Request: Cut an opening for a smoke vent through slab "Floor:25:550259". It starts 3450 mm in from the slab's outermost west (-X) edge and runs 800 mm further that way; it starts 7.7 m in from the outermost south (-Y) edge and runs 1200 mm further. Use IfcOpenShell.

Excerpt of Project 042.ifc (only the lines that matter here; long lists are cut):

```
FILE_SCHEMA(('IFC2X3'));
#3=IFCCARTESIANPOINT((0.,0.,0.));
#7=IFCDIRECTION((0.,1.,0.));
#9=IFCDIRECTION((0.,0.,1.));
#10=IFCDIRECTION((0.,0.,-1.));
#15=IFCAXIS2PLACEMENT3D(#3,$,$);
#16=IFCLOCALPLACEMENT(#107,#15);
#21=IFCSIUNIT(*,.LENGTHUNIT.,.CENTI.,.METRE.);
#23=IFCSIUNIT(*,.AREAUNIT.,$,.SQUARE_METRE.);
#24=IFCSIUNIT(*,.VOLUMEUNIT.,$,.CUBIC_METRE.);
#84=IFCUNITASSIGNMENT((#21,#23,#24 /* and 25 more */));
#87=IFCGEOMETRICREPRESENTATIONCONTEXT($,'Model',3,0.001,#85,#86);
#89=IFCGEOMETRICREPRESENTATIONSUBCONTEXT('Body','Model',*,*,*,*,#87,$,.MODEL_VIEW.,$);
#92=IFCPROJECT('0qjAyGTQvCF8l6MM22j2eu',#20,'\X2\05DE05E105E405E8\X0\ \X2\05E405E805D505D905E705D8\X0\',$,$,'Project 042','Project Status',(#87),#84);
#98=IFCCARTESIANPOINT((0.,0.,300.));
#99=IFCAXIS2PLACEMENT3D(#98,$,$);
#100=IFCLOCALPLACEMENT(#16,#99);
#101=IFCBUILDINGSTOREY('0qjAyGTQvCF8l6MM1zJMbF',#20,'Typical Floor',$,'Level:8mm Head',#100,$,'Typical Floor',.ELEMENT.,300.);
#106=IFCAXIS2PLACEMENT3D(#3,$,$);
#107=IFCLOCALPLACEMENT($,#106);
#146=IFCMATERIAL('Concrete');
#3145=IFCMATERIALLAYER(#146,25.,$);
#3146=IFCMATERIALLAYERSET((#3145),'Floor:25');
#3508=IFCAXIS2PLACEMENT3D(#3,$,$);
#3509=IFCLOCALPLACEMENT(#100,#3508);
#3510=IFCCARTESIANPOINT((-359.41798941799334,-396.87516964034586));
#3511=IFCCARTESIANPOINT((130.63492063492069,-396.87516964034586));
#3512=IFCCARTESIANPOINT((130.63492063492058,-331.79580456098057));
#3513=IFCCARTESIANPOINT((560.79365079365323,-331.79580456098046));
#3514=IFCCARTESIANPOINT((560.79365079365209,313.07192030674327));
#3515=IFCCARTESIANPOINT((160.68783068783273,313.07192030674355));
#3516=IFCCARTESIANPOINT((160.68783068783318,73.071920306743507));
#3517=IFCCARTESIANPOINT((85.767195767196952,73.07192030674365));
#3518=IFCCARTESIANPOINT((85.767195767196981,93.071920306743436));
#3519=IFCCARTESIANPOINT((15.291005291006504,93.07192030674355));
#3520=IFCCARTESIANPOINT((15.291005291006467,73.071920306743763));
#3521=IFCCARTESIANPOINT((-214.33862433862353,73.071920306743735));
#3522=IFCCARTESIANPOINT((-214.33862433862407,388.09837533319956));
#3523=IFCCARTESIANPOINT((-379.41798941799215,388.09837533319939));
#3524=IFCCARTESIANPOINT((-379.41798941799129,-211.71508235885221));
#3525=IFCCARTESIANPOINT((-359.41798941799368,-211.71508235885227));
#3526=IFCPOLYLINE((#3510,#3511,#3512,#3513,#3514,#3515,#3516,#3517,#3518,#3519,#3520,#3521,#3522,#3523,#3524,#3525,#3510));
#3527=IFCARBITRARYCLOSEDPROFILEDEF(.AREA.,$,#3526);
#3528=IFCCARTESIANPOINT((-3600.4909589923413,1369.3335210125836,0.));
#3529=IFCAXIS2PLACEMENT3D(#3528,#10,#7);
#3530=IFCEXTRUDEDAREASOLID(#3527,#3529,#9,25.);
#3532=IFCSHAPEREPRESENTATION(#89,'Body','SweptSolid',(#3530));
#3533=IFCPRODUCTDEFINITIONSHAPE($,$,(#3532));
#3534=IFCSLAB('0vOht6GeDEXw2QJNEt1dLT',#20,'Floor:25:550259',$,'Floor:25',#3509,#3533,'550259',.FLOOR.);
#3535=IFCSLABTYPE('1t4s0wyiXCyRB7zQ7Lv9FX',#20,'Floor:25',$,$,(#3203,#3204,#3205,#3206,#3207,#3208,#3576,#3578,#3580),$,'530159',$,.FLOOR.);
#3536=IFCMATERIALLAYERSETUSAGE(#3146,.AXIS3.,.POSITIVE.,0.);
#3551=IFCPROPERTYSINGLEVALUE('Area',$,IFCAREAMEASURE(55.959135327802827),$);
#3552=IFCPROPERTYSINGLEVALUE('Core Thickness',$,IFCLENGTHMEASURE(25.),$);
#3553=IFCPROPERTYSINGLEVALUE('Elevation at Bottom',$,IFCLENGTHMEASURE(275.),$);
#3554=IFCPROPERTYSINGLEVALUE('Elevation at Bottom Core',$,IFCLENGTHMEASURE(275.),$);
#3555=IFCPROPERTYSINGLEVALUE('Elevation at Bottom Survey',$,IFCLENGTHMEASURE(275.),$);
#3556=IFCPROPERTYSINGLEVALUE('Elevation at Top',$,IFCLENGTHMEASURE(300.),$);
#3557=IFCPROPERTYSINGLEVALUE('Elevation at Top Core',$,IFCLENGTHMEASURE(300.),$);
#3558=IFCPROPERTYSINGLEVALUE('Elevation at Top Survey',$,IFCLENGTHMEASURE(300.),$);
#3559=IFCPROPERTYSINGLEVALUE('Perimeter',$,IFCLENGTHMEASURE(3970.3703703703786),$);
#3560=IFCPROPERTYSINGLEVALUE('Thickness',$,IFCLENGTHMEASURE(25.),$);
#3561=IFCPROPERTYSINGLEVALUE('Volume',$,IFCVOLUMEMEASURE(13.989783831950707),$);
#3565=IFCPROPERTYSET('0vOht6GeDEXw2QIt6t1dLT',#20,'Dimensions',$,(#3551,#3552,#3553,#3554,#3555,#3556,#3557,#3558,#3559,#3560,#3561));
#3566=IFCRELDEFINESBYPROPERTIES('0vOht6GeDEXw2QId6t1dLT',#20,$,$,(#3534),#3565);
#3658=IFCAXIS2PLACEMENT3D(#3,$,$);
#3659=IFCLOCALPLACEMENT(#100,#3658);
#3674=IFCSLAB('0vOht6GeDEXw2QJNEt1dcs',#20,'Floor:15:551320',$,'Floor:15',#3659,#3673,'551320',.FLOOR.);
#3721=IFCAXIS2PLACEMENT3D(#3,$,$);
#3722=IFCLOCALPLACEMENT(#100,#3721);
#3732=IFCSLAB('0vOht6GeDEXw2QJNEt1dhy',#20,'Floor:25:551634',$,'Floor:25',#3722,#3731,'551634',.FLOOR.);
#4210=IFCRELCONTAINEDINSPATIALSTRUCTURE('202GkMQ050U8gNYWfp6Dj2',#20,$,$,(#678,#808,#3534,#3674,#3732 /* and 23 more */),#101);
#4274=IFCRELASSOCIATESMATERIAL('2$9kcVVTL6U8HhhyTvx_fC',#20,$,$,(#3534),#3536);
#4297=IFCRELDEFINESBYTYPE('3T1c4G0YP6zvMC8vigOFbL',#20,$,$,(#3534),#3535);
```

```python
import numpy as np
import ifcopenshell
import ifcopenshell.api.feature
import ifcopenshell.api.geometry
import ifcopenshell.api.pset
import ifcopenshell.api.root
import ifcopenshell.geom
import ifcopenshell.util.element
import ifcopenshell.util.placement
import ifcopenshell.util.representation
import ifcopenshell.util.shape
import ifcopenshell.util.unit

model = ifcopenshell.open("Project 042.ifc")
unit_scale = ifcopenshell.util.unit.calculate_unit_scale(model)
area_scale = ifcopenshell.util.unit.calculate_unit_scale(model, "AREAUNIT")
volume_scale = ifcopenshell.util.unit.calculate_unit_scale(model, "VOLUMEUNIT")
settings = ifcopenshell.geom.settings()


def volume(element):
    """Net volume in cubic metres, openings subtracted."""
    shape = ifcopenshell.geom.create_shape(settings, element)
    return ifcopenshell.util.shape.get_volume(shape.geometry)


slab = model.by_guid("0vOht6GeDEXw2QJNEt1dLT")
before = volume(slab)

# Extent in the slab's own axes, in metres. The edges named are its -X and -Y sides.
slab_shape = ifcopenshell.geom.create_shape(settings, slab)
vertices = ifcopenshell.util.shape.get_vertices(slab_shape.geometry)
x_min, y_min, bottom = vertices.min(axis=0)
top = vertices[:, 2].max()

opening = ifcopenshell.api.root.create_entity(model, ifc_class="IfcOpeningElement", name="Smoke vent opening")
context = ifcopenshell.util.representation.get_context(model, "Model", "Body", "MODEL_VIEW")
width, depth = 0.8, 1.2
outline = [(0.0, 0.0), (width, 0.0), (width, depth), (0.0, depth), (0.0, 0.0)]
# Overshoot both faces by 50 mm so the cut is clean.
shape = ifcopenshell.api.geometry.add_slab_representation(
    model, context=context, depth=top - bottom + 0.1, polyline=outline
)
ifcopenshell.api.geometry.assign_representation(model, product=opening, representation=shape)

matrix = ifcopenshell.util.placement.get_local_placement(slab.ObjectPlacement)
matrix[:, 3] = matrix @ np.append(np.array([x_min + 3.45, y_min + 7.7, bottom - 0.05]) / unit_scale, 1.0)
ifcopenshell.api.geometry.edit_object_placement(model, product=opening, matrix=matrix, is_si=False)
ifcopenshell.api.feature.add_feature(model, feature=opening, element=slab)

after = volume(slab)

# Update the slab's stored quantities.
pset = model.by_id(ifcopenshell.util.element.get_pset(slab, "Dimensions", should_inherit=False)["id"])
ifcopenshell.api.pset.edit_pset(model, pset=pset, properties={
    "Area": model.create_entity("IfcAreaMeasure", after / (top - bottom) / area_scale),
    "Volume": model.create_entity("IfcVolumeMeasure", after / volume_scale),
})

print(f"slab volume {before:.3f} -> {after:.3f} m3")

model.write("Project 042_rev.ifc")
```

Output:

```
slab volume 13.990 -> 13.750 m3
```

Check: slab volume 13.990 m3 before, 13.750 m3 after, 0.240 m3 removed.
